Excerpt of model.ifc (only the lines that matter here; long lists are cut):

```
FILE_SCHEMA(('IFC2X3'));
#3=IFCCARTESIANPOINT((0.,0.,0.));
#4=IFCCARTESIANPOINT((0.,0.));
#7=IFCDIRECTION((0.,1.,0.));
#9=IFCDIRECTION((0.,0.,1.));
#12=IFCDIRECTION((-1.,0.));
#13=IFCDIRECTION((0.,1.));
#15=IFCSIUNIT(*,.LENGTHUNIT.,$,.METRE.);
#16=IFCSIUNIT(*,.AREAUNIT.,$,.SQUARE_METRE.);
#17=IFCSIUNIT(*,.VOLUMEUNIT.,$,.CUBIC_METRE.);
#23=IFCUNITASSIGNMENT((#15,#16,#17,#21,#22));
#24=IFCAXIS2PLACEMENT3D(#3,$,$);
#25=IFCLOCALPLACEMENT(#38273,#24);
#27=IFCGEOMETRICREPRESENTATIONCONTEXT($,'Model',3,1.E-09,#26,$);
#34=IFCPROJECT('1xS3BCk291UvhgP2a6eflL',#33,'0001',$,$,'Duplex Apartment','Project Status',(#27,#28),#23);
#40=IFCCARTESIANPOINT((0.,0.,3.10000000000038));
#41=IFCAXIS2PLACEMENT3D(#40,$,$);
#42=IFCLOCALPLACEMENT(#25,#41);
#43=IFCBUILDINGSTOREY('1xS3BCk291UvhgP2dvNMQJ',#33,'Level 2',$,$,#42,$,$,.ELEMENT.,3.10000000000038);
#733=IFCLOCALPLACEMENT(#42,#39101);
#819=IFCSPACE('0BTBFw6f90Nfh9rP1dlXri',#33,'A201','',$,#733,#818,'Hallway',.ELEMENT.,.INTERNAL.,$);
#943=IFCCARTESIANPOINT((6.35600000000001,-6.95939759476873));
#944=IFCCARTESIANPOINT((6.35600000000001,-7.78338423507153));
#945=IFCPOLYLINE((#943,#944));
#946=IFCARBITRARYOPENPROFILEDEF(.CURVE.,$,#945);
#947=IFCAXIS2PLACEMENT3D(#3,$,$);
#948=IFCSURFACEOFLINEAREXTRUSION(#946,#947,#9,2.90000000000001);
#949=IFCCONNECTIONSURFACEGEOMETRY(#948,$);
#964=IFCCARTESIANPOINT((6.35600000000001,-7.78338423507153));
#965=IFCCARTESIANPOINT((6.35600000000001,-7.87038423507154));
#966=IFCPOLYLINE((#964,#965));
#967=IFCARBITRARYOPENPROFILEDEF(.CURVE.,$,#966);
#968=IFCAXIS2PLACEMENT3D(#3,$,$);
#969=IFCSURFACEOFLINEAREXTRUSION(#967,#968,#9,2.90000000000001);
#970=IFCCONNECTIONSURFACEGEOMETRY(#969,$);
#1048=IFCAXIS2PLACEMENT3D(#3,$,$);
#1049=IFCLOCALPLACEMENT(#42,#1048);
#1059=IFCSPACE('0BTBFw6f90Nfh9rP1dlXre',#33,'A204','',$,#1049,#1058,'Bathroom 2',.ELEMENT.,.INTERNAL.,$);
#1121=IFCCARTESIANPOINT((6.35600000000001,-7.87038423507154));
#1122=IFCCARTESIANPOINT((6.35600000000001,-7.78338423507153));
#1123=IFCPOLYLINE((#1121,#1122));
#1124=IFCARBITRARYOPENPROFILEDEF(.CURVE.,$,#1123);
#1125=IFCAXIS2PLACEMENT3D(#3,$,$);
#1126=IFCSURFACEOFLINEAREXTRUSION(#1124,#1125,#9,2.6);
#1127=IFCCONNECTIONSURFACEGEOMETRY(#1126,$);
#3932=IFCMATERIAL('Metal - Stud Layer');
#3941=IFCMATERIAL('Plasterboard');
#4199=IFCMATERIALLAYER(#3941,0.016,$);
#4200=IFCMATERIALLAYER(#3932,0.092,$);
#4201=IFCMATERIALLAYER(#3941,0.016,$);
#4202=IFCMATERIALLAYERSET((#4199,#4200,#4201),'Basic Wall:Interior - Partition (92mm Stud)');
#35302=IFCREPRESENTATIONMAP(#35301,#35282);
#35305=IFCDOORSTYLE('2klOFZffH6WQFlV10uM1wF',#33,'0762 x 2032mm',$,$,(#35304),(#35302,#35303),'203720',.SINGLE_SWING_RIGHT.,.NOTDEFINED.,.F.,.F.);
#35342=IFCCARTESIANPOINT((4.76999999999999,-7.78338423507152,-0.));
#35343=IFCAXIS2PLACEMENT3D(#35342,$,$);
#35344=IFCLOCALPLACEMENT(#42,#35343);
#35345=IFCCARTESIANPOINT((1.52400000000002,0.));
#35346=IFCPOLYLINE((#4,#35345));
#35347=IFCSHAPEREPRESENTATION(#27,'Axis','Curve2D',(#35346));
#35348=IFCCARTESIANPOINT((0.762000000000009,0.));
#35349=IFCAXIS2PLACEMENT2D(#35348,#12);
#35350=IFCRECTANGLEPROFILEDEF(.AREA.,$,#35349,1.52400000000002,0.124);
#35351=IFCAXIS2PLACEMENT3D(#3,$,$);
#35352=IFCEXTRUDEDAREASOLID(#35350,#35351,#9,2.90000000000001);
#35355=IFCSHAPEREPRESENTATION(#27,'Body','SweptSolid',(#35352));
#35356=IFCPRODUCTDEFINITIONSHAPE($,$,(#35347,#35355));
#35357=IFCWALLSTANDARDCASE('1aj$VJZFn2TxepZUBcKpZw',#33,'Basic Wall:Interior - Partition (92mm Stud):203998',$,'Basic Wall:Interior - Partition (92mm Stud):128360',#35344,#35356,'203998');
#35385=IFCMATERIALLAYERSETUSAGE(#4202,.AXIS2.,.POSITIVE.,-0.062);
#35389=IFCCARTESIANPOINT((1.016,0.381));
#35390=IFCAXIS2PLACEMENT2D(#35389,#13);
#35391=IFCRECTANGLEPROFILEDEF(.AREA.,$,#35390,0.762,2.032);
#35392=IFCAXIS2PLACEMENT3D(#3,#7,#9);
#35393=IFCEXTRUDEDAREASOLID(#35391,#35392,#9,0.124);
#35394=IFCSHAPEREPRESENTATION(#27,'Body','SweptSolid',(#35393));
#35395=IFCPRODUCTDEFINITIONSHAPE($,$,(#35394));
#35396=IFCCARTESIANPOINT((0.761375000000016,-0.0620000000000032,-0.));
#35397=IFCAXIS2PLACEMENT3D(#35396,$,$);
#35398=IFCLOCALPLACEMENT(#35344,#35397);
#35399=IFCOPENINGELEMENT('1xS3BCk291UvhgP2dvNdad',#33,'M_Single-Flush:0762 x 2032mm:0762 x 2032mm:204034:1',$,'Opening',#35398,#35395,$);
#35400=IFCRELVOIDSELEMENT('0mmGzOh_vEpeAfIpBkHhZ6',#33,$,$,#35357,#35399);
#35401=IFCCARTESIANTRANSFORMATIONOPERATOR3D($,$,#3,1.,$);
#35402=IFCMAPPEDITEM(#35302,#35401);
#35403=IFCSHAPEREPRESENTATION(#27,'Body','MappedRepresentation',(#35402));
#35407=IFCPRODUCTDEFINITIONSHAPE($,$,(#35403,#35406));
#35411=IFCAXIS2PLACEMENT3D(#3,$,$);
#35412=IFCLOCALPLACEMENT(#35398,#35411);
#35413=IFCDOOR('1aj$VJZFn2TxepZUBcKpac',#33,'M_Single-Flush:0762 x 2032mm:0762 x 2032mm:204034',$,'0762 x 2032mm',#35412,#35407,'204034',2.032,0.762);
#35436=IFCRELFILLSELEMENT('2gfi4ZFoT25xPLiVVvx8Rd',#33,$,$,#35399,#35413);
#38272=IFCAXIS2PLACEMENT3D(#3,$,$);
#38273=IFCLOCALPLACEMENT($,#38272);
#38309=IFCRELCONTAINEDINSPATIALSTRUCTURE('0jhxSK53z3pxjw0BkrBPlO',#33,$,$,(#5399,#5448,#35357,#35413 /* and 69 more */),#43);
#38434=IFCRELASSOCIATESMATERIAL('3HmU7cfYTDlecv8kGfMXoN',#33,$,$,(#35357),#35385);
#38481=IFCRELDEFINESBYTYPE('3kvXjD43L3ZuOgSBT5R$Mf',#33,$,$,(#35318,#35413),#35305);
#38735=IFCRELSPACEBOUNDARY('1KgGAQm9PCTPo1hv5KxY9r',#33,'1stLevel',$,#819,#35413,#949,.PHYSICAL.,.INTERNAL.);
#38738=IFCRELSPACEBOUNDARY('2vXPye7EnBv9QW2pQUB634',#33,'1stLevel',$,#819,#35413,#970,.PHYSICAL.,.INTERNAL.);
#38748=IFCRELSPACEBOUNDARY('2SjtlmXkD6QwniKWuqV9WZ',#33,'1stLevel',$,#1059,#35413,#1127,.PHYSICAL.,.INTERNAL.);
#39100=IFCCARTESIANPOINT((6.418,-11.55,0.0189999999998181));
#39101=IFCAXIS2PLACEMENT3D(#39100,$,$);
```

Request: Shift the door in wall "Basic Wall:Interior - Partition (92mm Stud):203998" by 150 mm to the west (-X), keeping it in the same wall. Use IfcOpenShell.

```python
import numpy as np
import ifcopenshell
import ifcopenshell.api.geometry
import ifcopenshell.util.placement
import ifcopenshell.util.unit

model = ifcopenshell.open("model.ifc")
unit_scale = ifcopenshell.util.unit.calculate_unit_scale(model)

door = model.by_guid("1aj$VJZFn2TxepZUBcKpac")
opening = door.FillsVoids[0].RelatingOpeningElement
wall = opening.VoidsElements[0].RelatingBuildingElement

wall_matrix = ifcopenshell.util.placement.get_local_placement(wall.ObjectPlacement)
shift = wall_matrix[:3, 0] * -0.15 / unit_scale
before = ifcopenshell.util.placement.get_local_placement(door.ObjectPlacement)[:3, 3].copy()

# The door is placed relative to its opening, so it follows when the opening moves.
matrix = ifcopenshell.util.placement.get_local_placement(opening.ObjectPlacement)
matrix[:3, 3] += shift
ifcopenshell.api.geometry.edit_object_placement(
    model, product=opening, matrix=matrix, is_si=False, should_transform_children=True
)

# Space boundary surfaces are stored in each space's coordinates; move them too.
for rel in door.ProvidesBoundaries:
    if not rel.ConnectionGeometry:
        continue
    surface = rel.ConnectionGeometry.SurfaceOnRelatingElement
    space_matrix = ifcopenshell.util.placement.get_local_placement(rel.RelatingSpace.ObjectPlacement)
    point = np.array(surface.Position.Location.Coordinates) + space_matrix[:3, :3].T @ shift
    surface.Position = model.createIfcAxis2Placement3D(
        model.createIfcCartesianPoint(point.tolist()), surface.Position.Axis, surface.Position.RefDirection
    )

after = ifcopenshell.util.placement.get_local_placement(door.ObjectPlacement)[:3, 3]
print("door moved by", (after - before).round(3) + 0.0)

model.write("model-out.ifc")
```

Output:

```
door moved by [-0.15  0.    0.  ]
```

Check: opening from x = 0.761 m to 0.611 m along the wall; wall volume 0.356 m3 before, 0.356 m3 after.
